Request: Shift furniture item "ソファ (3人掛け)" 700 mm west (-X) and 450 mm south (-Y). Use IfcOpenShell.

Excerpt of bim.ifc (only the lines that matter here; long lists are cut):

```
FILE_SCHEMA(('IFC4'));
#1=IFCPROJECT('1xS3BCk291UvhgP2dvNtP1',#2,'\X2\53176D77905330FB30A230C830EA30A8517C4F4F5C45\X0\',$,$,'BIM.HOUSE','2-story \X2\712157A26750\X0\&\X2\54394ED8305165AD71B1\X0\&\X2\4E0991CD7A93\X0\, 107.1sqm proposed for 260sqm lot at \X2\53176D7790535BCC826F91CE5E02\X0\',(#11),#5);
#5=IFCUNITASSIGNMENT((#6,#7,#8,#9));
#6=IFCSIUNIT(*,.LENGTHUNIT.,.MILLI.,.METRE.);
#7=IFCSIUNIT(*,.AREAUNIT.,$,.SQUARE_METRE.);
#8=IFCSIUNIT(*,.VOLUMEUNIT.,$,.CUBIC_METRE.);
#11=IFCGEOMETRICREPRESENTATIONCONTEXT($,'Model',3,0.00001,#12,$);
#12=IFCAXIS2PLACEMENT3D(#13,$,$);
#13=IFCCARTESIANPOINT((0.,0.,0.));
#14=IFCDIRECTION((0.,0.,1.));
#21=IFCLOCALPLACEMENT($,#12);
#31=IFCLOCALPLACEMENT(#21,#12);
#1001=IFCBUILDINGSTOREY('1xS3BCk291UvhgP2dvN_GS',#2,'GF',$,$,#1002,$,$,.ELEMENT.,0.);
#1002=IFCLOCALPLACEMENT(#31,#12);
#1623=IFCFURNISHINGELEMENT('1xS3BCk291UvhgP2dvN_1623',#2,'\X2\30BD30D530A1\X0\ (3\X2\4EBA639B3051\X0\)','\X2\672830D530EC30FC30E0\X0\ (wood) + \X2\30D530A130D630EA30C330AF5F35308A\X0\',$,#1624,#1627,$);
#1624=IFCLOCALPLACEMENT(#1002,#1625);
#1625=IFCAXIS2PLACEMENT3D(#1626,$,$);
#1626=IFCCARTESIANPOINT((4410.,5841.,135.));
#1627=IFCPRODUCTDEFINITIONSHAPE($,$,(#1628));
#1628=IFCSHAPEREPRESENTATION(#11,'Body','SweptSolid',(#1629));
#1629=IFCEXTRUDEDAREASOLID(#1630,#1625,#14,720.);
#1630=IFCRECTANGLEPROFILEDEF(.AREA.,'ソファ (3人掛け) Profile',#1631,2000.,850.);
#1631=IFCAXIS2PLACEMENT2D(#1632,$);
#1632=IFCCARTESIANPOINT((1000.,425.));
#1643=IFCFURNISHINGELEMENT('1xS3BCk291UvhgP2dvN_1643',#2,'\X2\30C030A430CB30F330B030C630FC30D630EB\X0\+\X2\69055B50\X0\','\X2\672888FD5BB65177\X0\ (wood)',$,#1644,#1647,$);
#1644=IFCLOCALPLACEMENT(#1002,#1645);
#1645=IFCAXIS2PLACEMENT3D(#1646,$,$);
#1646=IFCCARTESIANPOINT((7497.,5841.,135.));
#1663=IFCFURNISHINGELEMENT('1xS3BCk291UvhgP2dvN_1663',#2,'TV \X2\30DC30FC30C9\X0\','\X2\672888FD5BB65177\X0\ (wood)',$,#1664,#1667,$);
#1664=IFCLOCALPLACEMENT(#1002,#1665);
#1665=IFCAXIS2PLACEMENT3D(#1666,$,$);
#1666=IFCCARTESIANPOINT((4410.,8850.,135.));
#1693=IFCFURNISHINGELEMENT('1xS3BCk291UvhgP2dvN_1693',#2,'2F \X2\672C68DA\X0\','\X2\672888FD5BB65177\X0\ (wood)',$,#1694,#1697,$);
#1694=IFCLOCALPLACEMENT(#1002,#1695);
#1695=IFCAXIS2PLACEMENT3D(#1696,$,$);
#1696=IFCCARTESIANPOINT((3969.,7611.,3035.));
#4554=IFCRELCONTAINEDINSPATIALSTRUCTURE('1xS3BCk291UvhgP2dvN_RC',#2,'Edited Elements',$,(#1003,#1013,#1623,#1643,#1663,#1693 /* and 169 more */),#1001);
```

```python
import ifcopenshell
import ifcopenshell.api.geometry
import ifcopenshell.util.placement
import ifcopenshell.util.unit

model = ifcopenshell.open("bim.ifc")
unit_scale = ifcopenshell.util.unit.calculate_unit_scale(model)

item = model.by_guid("1xS3BCk291UvhgP2dvN_1623")
matrix = ifcopenshell.util.placement.get_local_placement(item.ObjectPlacement)
matrix[0, 3] -= 0.7 / unit_scale
matrix[1, 3] -= 0.45 / unit_scale
ifcopenshell.api.geometry.edit_object_placement(model, product=item, matrix=matrix, is_si=False)

print(ifcopenshell.util.placement.get_local_placement(item.ObjectPlacement).round(3) + 0.0)

model.write("bim_rev.ifc")
```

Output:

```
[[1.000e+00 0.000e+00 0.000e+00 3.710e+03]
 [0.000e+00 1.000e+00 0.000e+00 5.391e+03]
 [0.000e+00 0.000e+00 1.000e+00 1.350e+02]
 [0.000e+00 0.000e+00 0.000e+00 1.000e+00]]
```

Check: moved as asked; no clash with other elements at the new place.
